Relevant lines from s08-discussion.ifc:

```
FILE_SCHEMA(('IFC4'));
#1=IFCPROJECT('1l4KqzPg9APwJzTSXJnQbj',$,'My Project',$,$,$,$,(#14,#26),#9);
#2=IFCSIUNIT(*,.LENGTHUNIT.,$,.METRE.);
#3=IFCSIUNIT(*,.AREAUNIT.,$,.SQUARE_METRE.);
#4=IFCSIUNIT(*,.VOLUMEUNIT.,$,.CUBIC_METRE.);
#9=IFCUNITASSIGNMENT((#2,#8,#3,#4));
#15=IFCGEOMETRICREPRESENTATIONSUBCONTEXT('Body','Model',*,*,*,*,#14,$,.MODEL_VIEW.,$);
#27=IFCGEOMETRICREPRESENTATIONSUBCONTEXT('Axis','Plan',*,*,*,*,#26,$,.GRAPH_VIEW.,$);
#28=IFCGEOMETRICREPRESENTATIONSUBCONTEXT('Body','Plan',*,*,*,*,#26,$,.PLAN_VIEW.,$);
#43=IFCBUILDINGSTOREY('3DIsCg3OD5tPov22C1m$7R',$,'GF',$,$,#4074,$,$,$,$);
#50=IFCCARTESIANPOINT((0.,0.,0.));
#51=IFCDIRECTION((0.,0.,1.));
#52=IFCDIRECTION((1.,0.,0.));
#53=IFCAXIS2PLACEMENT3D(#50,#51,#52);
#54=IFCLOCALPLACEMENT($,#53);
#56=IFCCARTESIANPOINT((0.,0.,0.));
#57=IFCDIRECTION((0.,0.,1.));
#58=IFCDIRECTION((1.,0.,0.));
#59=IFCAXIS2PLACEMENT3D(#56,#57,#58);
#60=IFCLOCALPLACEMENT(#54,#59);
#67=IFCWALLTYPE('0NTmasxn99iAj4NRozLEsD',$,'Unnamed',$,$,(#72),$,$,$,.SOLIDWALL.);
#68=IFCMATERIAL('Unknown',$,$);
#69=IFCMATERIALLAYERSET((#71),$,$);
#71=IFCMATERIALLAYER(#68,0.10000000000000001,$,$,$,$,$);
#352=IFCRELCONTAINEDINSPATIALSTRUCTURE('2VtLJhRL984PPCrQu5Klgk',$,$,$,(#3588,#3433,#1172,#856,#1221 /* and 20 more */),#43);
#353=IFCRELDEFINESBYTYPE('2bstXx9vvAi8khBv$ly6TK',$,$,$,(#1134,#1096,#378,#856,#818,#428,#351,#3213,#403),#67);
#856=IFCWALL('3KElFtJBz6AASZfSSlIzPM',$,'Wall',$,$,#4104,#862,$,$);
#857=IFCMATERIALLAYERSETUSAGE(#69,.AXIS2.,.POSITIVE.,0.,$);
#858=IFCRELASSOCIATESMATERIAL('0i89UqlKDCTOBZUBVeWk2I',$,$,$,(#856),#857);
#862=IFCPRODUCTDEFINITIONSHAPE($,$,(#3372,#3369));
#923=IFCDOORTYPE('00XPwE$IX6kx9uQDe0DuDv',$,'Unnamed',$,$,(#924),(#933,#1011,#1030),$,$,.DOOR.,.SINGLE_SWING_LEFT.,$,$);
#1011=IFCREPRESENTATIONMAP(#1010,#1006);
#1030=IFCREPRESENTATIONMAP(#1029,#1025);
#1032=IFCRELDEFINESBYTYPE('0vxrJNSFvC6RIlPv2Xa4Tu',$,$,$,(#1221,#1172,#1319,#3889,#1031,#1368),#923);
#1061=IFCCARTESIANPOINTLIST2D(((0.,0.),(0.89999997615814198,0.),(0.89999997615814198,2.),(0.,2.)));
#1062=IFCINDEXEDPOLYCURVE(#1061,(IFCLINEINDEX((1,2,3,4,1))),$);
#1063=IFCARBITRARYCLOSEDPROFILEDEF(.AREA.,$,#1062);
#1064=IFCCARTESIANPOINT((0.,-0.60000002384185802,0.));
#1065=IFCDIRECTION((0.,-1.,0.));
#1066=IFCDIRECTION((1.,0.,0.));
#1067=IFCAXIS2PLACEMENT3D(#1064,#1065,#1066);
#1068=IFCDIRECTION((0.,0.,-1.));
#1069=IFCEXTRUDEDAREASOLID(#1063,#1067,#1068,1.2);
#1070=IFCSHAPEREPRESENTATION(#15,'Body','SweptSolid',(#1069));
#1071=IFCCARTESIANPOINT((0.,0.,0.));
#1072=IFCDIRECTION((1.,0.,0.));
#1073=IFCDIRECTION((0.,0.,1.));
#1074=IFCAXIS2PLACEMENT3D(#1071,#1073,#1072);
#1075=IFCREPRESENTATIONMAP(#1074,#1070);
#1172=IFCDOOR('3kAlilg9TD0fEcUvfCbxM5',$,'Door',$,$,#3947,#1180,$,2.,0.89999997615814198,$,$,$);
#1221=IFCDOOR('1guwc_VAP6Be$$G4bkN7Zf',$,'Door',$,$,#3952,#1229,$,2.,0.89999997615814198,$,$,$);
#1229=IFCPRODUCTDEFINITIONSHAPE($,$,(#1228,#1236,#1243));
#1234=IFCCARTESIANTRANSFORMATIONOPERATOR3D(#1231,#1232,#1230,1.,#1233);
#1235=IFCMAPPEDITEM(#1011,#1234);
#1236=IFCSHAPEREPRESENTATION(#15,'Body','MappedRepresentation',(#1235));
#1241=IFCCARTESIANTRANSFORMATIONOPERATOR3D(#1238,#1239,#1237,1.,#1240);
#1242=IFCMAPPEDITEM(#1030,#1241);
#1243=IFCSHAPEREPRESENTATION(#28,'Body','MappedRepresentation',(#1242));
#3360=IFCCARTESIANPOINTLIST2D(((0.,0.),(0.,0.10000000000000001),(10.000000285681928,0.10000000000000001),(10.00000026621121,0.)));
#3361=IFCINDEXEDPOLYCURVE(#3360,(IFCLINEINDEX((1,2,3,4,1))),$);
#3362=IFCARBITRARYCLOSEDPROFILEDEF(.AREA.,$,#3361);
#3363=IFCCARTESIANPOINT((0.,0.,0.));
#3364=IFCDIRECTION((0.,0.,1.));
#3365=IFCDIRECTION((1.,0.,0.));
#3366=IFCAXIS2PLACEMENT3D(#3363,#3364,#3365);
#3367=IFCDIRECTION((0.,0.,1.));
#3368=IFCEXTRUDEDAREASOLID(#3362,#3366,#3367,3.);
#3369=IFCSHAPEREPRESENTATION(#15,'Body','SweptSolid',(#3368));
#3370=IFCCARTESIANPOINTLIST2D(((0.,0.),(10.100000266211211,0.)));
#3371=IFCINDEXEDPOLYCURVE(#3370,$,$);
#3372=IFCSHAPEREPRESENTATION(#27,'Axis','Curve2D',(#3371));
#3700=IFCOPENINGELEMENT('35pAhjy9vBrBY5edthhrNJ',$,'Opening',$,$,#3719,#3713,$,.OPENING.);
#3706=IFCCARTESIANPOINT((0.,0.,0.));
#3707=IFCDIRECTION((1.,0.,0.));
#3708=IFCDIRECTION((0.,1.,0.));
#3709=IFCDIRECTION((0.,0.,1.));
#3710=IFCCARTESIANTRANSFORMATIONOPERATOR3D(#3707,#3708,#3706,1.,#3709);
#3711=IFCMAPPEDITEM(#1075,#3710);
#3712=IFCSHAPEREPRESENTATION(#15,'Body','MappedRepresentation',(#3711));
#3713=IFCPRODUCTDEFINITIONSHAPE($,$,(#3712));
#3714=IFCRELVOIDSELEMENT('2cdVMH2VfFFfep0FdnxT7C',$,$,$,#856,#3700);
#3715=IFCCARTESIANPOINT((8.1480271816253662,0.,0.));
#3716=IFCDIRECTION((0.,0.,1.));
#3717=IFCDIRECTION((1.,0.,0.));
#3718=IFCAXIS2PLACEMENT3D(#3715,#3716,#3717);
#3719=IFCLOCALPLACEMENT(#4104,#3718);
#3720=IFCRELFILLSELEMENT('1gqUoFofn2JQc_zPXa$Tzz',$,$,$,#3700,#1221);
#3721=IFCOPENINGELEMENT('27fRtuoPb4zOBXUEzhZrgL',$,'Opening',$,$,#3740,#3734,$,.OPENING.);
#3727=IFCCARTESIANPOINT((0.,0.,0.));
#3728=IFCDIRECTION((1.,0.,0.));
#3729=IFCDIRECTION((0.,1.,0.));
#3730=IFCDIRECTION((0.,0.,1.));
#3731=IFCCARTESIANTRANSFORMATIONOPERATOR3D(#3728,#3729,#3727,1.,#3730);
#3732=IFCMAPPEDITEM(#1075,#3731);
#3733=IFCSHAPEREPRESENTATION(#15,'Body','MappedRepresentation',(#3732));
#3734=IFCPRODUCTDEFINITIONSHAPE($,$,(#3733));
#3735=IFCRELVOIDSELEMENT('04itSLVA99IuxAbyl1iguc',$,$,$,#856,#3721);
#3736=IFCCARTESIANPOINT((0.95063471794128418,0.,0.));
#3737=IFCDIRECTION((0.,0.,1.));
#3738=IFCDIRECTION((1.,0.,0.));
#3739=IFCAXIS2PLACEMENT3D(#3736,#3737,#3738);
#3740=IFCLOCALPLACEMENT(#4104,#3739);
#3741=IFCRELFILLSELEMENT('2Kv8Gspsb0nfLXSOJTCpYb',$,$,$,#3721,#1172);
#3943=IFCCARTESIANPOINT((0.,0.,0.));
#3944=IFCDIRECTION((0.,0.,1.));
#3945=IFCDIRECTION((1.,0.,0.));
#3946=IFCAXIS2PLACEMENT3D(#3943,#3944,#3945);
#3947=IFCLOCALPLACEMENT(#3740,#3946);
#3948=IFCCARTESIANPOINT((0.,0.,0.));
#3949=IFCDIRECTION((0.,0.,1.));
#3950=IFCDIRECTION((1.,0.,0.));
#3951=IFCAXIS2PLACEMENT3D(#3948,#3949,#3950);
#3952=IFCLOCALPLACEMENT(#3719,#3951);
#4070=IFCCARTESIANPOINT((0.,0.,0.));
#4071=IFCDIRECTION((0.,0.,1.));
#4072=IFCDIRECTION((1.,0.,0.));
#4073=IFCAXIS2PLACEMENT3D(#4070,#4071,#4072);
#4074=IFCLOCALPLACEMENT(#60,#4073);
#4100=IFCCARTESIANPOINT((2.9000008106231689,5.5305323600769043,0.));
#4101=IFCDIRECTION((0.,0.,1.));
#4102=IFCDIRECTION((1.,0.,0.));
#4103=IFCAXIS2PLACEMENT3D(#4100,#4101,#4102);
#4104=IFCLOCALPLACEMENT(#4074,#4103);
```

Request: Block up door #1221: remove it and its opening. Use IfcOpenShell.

```python
import ifcopenshell
import ifcopenshell.api.feature
import ifcopenshell.api.root
import ifcopenshell.geom
import ifcopenshell.util.shape

model = ifcopenshell.open("s08-discussion.ifc")
settings = ifcopenshell.geom.settings()


def volume(element):
    """Net volume in cubic metres, openings subtracted."""
    shape = ifcopenshell.geom.create_shape(settings, element)
    return ifcopenshell.util.shape.get_volume(shape.geometry)


door = model.by_id(1221)
opening = door.FillsVoids[0].RelatingOpeningElement
wall = opening.VoidsElements[0].RelatingBuildingElement
before = volume(wall)

ifcopenshell.api.root.remove_product(model, product=door)
ifcopenshell.api.feature.remove_feature(model, feature=opening)

after = volume(wall)

print(f"wall volume {before:.3f} -> {after:.3f} m3")

model.write("s08-discussion-out.ifc")
```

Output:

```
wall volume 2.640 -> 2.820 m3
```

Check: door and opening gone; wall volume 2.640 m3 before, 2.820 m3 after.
